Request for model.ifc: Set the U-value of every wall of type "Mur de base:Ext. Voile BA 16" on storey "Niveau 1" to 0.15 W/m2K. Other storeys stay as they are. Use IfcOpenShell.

First a look at what the model holds.

```python
import ifcopenshell
import ifcopenshell.util.element

model = ifcopenshell.open("model.ifc")
print(model.schema)
storey = next(s for s in model.by_type("IfcBuildingStorey") if s.Name == "Niveau 1")
walls = [e for e in ifcopenshell.util.element.get_decomposition(storey) if e.is_a("IfcWall")]
seen = {}
for e in walls:
    element_type = ifcopenshell.util.element.get_type(e)
    key = (element_type.Name if element_type != e and element_type else None, ifcopenshell.util.element.get_pset(e, "Pset_WallCommon", "ThermalTransmittance"))
    seen[key] = seen.get(key, 0) + 1
for (name, value), count in sorted(seen.items(), key=str):
    print(count, "x", name, "|", value)
```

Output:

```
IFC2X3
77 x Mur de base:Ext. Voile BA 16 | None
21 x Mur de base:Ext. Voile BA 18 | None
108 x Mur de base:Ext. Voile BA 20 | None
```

```python
import ifcopenshell
import ifcopenshell.api.pset
import ifcopenshell.util.element

model = ifcopenshell.open("model.ifc")

storey = next(s for s in model.by_type("IfcBuildingStorey") if s.Name == "Niveau 1")
walls = [e for e in ifcopenshell.util.element.get_decomposition(storey) if e.is_a("IfcWall")]

count = 0
for e in walls:
    element_type = ifcopenshell.util.element.get_type(e)
    if element_type in (None, e) or element_type.Name != "Mur de base:Ext. Voile BA 16":
        continue
    # add_pset returns the element's existing set when there is one.
    pset = ifcopenshell.api.pset.add_pset(model, product=e, name="Pset_WallCommon")
    ifcopenshell.api.pset.edit_pset(model, pset=pset, properties={"ThermalTransmittance": 0.15})
    count += 1

print(count, "walls updated")

model.write("model-out.ifc")
```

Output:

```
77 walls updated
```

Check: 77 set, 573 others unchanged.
